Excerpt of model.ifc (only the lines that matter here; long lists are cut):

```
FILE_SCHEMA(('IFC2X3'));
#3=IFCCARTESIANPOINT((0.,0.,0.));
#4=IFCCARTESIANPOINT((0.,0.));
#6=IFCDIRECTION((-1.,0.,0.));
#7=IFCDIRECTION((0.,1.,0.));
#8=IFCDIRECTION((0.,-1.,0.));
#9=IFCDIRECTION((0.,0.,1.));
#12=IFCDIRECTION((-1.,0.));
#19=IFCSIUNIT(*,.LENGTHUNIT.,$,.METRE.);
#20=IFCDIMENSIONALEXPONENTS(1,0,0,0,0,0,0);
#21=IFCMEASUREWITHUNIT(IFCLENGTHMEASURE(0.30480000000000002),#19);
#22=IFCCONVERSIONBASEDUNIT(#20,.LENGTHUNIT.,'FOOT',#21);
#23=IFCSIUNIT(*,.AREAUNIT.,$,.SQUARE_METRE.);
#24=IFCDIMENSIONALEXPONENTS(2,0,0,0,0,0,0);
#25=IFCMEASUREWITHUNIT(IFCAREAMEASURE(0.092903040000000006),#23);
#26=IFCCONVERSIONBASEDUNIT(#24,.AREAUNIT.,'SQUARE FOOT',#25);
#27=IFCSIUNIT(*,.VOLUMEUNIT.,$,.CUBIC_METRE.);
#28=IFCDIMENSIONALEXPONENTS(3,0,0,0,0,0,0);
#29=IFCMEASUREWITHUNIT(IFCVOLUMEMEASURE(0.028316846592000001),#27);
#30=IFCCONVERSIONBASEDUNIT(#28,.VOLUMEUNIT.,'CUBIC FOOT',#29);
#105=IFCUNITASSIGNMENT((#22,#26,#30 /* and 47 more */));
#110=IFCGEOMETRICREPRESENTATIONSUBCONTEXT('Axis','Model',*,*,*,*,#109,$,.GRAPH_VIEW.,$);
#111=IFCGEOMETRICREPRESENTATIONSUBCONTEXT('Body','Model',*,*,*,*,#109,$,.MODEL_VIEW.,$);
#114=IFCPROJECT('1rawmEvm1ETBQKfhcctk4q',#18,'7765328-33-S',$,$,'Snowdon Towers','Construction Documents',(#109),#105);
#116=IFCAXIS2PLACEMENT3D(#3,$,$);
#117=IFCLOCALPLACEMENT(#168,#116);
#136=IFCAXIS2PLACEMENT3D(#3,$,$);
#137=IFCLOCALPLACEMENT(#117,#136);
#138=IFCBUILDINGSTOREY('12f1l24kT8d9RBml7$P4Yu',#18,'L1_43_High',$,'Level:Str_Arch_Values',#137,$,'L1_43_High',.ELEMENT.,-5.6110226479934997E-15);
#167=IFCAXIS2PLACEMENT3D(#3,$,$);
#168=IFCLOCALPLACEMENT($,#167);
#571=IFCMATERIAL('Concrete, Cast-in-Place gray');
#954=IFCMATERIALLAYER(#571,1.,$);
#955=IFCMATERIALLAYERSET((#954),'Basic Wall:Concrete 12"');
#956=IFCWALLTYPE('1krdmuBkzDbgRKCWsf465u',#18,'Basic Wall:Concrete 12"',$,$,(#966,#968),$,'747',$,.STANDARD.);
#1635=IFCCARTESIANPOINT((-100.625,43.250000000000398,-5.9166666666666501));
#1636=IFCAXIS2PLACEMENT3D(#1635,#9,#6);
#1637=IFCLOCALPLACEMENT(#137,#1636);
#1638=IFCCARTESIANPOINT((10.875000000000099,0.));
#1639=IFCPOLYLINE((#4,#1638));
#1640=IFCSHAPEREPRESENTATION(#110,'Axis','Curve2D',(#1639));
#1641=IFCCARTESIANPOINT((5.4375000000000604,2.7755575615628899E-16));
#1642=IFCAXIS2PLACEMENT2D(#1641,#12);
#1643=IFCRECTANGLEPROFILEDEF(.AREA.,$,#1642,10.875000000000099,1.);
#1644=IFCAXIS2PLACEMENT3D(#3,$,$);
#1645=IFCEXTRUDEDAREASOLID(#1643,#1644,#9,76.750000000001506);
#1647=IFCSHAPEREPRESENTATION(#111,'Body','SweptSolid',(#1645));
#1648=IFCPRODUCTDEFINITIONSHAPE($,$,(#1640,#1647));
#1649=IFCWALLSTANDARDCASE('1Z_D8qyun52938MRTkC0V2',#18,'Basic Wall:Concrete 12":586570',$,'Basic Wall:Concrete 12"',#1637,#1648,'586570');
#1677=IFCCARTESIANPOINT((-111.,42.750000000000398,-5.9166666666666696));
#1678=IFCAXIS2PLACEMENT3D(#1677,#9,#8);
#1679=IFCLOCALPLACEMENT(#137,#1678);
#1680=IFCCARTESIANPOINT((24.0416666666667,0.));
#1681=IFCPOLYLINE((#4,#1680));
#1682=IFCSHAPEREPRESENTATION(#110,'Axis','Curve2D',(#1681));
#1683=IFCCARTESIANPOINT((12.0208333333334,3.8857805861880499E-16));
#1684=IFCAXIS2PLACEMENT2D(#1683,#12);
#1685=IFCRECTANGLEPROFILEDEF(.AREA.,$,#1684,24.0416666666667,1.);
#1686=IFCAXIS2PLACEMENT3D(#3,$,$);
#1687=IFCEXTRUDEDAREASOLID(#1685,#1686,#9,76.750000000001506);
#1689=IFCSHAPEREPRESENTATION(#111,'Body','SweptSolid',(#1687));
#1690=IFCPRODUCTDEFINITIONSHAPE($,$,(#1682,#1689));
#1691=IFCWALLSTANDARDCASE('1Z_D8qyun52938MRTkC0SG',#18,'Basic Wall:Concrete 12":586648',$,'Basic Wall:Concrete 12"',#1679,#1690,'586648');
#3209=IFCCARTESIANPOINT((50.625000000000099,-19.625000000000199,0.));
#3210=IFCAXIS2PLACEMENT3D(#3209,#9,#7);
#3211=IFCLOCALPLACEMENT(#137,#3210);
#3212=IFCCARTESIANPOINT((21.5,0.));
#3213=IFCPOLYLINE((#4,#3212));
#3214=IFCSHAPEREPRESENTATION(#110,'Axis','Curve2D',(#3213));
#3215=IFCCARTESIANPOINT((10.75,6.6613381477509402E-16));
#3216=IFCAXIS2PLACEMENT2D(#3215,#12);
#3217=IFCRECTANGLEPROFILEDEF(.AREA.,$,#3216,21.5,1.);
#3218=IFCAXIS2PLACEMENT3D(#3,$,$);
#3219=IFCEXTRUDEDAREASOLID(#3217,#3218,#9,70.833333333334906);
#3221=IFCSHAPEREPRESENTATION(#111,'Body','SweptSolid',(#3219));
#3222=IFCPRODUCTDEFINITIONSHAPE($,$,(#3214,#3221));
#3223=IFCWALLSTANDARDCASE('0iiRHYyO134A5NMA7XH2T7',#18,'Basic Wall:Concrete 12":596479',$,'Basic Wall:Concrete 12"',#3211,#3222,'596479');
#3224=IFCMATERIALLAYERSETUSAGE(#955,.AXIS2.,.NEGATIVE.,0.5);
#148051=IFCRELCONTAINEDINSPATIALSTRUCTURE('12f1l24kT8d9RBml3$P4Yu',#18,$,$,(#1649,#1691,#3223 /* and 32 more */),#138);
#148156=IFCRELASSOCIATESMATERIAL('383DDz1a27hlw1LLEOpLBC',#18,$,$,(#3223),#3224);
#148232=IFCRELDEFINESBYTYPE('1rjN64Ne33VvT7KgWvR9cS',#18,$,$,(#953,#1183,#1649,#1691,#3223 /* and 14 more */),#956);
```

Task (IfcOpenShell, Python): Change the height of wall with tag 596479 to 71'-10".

```python
import ifcopenshell
import ifcopenshell.geom
import ifcopenshell.util.representation
import ifcopenshell.util.shape
import ifcopenshell.util.unit

model = ifcopenshell.open("model.ifc")
unit_scale = ifcopenshell.util.unit.calculate_unit_scale(model)
settings = ifcopenshell.geom.settings()


def volume(element):
    """Net volume in cubic metres, openings subtracted."""
    shape = ifcopenshell.geom.create_shape(settings, element)
    return ifcopenshell.util.shape.get_volume(shape.geometry)


wall = model.by_id(3223)
before = volume(wall)

body = ifcopenshell.util.representation.get_representation(wall, "Model", "Body")
solid = body.Items[0]
old_height = solid.Depth
solid.Depth = 862 * 0.0254 / unit_scale
after = volume(wall)

print(f"height {old_height:g} -> {solid.Depth:g}, volume {before:.3f} -> {after:.3f} m3")

model.write("model_updated.ifc")
```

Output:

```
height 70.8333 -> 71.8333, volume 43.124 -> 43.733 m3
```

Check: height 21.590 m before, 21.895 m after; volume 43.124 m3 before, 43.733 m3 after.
